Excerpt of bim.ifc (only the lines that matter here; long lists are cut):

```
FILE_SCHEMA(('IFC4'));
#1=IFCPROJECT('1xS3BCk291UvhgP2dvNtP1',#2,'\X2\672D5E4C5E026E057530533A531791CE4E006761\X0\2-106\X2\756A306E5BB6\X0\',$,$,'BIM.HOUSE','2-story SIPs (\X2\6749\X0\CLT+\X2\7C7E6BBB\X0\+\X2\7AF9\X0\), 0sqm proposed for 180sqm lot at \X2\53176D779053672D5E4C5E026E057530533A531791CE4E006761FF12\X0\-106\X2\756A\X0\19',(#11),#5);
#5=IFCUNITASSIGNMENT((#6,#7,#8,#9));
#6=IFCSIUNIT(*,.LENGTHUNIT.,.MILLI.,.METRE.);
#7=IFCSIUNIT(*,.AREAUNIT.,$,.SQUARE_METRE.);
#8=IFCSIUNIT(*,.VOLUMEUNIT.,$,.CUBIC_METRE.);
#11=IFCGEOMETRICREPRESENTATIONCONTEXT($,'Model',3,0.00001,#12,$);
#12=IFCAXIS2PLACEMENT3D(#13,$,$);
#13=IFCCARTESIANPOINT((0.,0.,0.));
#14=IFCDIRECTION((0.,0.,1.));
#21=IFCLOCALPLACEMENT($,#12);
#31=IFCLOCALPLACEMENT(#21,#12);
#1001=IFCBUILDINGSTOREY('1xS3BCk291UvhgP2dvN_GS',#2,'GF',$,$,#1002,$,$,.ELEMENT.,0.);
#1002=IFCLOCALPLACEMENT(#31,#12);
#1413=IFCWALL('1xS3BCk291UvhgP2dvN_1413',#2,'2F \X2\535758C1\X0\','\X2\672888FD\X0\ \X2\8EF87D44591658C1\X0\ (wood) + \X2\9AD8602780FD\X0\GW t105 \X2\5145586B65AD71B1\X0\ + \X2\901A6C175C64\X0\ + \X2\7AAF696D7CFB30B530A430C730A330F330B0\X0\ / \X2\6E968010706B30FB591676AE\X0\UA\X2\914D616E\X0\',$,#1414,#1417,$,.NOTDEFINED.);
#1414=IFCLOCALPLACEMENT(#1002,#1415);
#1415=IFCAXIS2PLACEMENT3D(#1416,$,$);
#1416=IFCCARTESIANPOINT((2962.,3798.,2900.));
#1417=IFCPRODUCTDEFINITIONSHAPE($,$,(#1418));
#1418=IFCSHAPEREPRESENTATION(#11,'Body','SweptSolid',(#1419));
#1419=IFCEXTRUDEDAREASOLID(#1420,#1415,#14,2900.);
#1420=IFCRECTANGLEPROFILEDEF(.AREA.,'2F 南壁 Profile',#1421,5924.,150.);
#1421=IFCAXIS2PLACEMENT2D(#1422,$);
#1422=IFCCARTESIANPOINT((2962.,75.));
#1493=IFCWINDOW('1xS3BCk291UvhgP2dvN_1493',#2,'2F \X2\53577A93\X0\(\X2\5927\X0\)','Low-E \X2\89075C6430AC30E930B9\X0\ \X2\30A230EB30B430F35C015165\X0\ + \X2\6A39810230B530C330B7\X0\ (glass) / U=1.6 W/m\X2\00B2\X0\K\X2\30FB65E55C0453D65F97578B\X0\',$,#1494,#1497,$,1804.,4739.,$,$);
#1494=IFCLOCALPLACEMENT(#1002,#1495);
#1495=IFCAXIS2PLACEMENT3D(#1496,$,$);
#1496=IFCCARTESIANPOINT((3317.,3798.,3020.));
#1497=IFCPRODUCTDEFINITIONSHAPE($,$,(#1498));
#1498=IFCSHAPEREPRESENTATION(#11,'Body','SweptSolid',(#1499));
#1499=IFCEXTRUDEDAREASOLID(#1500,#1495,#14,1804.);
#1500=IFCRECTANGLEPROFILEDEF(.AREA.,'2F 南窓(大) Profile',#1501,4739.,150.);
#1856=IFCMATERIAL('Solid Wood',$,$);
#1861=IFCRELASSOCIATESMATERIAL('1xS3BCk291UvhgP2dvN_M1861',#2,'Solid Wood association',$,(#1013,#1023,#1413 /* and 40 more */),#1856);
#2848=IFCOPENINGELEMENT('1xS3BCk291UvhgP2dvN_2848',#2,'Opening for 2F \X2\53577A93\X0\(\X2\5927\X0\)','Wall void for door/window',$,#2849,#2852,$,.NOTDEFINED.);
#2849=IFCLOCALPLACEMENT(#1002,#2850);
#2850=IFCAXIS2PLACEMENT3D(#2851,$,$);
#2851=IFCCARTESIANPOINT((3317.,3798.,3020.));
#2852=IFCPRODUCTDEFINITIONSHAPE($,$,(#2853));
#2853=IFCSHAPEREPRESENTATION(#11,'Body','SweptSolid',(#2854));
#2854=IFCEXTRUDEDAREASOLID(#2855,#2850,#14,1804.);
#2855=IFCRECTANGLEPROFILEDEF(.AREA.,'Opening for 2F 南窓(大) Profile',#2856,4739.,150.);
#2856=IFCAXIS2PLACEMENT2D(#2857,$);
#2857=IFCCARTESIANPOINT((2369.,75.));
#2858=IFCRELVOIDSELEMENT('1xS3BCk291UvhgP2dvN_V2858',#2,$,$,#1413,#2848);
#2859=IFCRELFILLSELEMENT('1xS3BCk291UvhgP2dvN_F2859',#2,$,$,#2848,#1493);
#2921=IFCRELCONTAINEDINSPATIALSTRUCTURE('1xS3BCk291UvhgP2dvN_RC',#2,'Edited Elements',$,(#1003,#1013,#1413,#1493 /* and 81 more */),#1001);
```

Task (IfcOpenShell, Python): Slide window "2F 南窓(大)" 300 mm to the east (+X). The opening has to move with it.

```python
import ifcopenshell
import ifcopenshell.api.geometry
import ifcopenshell.util.placement

model = ifcopenshell.open("bim.ifc")

window = model.by_guid("1xS3BCk291UvhgP2dvN_1493")
opening = window.FillsVoids[0].RelatingOpeningElement
wall = opening.VoidsElements[0].RelatingBuildingElement

wall_matrix = ifcopenshell.util.placement.get_local_placement(wall.ObjectPlacement)
shift = wall_matrix[:3, 0] * 300.0
before = ifcopenshell.util.placement.get_local_placement(window.ObjectPlacement)[:3, 3].copy()

# The window is not placed relative to its opening, so move both.
for product in (opening, window):
    matrix = ifcopenshell.util.placement.get_local_placement(product.ObjectPlacement)
    matrix[:3, 3] += shift
    ifcopenshell.api.geometry.edit_object_placement(model, product=product, matrix=matrix, is_si=False)

after = ifcopenshell.util.placement.get_local_placement(window.ObjectPlacement)[:3, 3]
print("window moved by", (after - before).round(3) + 0.0)

model.write("bim_rev.ifc")
```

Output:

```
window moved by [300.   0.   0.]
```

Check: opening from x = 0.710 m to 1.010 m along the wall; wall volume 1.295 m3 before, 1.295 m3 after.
